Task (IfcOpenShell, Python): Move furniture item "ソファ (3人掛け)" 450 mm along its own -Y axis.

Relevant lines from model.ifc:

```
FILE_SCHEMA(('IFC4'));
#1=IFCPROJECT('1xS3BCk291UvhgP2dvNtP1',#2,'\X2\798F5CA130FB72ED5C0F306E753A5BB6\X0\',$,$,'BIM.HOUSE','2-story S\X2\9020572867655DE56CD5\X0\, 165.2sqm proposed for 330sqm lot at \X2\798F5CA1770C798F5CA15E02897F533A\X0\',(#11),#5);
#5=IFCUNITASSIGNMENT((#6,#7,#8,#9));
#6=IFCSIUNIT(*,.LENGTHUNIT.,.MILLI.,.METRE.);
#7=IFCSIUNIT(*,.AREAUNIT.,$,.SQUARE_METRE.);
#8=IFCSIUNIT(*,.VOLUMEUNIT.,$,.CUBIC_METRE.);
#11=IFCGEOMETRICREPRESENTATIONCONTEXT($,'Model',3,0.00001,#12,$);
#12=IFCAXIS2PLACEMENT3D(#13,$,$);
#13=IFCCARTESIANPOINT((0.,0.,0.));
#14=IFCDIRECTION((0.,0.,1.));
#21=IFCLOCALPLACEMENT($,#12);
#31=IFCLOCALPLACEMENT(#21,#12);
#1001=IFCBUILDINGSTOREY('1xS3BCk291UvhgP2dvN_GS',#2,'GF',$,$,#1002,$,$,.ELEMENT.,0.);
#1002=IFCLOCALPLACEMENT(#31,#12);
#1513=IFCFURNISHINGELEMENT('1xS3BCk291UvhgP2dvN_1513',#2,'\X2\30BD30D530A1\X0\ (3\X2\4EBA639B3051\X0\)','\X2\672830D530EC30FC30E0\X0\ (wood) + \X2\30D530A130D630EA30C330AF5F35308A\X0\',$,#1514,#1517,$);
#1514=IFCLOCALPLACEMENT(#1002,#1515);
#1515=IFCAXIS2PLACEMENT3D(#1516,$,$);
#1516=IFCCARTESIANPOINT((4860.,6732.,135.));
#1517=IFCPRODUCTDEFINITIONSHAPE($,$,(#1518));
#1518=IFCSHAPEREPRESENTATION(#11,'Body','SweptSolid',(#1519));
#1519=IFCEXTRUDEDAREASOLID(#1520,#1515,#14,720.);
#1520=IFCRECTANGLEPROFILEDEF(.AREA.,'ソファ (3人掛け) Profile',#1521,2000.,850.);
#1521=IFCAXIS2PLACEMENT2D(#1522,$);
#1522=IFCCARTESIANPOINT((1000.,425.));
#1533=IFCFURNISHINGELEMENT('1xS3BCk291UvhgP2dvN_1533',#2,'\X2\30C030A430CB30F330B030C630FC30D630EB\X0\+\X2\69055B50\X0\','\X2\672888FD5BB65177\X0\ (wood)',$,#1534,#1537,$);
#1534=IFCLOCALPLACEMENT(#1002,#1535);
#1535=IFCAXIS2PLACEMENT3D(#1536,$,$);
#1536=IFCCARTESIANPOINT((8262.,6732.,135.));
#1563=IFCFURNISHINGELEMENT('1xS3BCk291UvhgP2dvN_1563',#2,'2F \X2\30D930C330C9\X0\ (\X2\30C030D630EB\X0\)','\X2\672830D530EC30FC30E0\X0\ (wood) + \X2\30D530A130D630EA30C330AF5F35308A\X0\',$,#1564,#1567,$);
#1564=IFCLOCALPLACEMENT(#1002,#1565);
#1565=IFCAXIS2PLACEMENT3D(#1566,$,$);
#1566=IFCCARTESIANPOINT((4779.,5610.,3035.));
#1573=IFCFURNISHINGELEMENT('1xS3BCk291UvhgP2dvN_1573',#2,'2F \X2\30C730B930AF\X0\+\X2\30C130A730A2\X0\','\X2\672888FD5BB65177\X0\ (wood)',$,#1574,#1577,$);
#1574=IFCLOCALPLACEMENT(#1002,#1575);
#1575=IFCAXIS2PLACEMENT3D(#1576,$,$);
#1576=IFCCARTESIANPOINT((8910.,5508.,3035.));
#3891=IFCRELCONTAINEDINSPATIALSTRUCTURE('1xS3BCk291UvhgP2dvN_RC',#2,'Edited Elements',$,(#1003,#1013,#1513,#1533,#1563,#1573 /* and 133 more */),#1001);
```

```python
import ifcopenshell
import ifcopenshell.api.geometry
import ifcopenshell.util.placement

model = ifcopenshell.open("model.ifc")

item = model.by_guid("1xS3BCk291UvhgP2dvN_1513")
matrix = ifcopenshell.util.placement.get_local_placement(item.ObjectPlacement)
matrix[:3, 3] -= matrix[:3, 1] * 450.0
ifcopenshell.api.geometry.edit_object_placement(model, product=item, matrix=matrix, is_si=False)

print(ifcopenshell.util.placement.get_local_placement(item.ObjectPlacement).round(3) + 0.0)

model.write("model_rev.ifc")
```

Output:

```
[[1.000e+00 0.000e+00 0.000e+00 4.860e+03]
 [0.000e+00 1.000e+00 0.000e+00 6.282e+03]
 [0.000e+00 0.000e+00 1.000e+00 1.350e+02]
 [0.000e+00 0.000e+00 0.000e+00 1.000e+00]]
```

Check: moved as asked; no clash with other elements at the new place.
